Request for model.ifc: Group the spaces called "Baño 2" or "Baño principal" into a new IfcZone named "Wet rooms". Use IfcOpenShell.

First a look at what the model holds.

```python
import ifcopenshell

model = ifcopenshell.open("model.ifc")
print(model.schema)
seen = {}
for space in model.by_type("IfcSpace"):
    seen[space.LongName] = seen.get(space.LongName, 0) + 1
for name, count in sorted(seen.items(), key=str):
    print(count, "x", name)
print("zones:", [z.Name for z in model.by_type("IfcZone")][:20])
```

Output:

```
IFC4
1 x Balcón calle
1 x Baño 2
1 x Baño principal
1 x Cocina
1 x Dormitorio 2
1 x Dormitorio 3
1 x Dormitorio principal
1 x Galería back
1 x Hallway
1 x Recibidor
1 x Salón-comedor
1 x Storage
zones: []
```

```python
import ifcopenshell
import ifcopenshell.api.group
import ifcopenshell.api.root

model = ifcopenshell.open("model.ifc")

names = {"Baño 2", "Baño principal"}
spaces = [s for s in model.by_type("IfcSpace") if s.LongName in names]

zone = ifcopenshell.api.root.create_entity(model, ifc_class="IfcZone", name="Wet rooms")
ifcopenshell.api.group.assign_group(model, products=spaces, group=zone)
print(len(spaces), "spaces in", zone.Name)

model.write("model_edited.ifc")
```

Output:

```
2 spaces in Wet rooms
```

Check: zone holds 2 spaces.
